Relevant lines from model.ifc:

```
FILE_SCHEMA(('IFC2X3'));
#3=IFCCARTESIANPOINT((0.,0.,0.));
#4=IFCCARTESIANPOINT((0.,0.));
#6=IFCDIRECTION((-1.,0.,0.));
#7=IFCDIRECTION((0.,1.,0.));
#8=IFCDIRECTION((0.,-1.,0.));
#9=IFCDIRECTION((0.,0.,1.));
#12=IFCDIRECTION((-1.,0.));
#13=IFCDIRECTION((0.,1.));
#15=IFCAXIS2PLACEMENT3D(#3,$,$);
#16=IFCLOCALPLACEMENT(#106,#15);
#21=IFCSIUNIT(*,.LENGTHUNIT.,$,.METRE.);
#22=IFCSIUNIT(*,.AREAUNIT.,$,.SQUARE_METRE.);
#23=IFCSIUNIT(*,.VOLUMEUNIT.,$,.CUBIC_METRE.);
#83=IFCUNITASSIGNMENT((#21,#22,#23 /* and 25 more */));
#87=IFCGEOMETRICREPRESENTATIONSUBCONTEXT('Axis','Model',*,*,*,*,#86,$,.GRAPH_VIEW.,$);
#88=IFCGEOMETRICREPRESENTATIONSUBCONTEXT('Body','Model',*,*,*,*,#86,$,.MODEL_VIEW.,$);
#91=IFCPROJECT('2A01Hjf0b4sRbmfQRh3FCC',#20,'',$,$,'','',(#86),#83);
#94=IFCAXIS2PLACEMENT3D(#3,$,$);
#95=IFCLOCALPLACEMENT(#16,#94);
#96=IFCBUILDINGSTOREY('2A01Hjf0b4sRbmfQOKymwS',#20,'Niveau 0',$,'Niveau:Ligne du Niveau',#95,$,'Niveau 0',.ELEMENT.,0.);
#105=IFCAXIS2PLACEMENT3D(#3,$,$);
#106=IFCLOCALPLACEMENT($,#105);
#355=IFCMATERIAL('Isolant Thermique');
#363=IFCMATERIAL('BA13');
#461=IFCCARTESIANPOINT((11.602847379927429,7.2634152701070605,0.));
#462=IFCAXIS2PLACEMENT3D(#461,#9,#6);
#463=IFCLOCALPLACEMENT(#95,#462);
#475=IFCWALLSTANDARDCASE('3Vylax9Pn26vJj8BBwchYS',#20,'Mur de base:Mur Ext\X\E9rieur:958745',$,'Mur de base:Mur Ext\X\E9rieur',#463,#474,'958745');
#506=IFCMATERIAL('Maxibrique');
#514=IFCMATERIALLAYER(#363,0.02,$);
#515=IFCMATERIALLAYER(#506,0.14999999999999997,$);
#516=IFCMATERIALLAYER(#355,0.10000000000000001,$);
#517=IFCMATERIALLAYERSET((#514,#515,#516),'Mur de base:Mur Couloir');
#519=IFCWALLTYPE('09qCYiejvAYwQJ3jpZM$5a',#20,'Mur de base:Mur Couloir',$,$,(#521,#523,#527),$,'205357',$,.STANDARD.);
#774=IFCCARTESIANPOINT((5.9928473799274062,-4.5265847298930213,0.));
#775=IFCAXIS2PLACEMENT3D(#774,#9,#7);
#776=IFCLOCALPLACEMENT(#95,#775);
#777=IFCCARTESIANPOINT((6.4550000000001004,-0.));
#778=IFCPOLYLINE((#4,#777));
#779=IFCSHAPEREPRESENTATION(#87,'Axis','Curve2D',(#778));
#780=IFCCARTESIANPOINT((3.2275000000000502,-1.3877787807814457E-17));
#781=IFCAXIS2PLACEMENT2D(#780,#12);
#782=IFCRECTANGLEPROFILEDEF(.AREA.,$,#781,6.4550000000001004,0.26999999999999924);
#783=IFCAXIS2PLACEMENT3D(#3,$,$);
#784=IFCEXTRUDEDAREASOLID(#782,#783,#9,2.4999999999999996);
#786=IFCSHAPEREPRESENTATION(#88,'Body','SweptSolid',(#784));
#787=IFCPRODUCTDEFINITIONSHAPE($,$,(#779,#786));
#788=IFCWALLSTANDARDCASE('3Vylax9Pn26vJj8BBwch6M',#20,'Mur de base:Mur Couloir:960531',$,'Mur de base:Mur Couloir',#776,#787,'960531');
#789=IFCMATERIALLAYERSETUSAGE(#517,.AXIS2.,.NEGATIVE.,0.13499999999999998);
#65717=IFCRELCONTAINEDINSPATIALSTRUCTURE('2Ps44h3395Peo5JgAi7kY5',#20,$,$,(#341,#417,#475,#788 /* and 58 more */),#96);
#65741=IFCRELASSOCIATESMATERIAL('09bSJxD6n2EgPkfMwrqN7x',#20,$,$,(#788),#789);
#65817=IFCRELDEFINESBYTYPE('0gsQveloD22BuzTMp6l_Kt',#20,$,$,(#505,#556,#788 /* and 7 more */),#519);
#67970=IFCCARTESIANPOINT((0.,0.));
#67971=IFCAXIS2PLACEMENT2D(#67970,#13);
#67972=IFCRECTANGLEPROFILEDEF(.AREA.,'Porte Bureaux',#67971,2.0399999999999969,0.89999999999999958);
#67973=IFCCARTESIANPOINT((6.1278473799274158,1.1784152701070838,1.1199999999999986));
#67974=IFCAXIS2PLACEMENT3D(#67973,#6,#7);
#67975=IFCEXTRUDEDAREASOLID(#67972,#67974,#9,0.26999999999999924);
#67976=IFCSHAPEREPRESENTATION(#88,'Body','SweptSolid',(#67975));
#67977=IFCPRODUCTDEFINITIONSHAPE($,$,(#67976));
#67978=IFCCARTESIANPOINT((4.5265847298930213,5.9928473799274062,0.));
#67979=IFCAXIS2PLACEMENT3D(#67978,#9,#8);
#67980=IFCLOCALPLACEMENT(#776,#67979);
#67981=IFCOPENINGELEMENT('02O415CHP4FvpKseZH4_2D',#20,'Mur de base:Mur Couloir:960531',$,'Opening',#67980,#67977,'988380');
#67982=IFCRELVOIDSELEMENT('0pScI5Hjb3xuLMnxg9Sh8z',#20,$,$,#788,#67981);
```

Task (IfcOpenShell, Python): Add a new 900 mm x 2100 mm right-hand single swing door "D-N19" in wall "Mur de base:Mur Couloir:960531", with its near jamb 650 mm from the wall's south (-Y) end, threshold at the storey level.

```python
import numpy as np
import ifcopenshell
import ifcopenshell.api.feature
import ifcopenshell.api.geometry
import ifcopenshell.api.root
import ifcopenshell.api.spatial
import ifcopenshell.api.type
import ifcopenshell.geom
import ifcopenshell.util.element
import ifcopenshell.util.placement
import ifcopenshell.util.representation
import ifcopenshell.util.shape
import ifcopenshell.util.unit

model = ifcopenshell.open("model.ifc")
unit_scale = ifcopenshell.util.unit.calculate_unit_scale(model)
settings = ifcopenshell.geom.settings()


def volume(element):
    """Net volume in cubic metres, openings subtracted."""
    shape = ifcopenshell.geom.create_shape(settings, element)
    return ifcopenshell.util.shape.get_volume(shape.geometry)


wall = model.by_id(788)
storey = ifcopenshell.util.element.get_container(wall, ifc_class="IfcBuildingStorey")
context = ifcopenshell.util.representation.get_context(model, "Model", "Body", "MODEL_VIEW")
before = volume(wall)

width, height, from_end, sill = 0.9, 2.1, 0.65, 0.0  # metres

# The wall runs along its own X axis, and the end named is its -X end.
wall_shape = ifcopenshell.geom.create_shape(settings, wall)
x, y, z = ifcopenshell.util.shape.get_vertices(wall_shape.geometry).T
start = x.min() + from_end
face, thickness = float(y.min()), float(y.max() - y.min())
wall_matrix = ifcopenshell.util.placement.get_local_placement(wall.ObjectPlacement)
level = ifcopenshell.util.placement.get_local_placement(storey.ObjectPlacement)[2, 3]


def in_wall(x, y):
    """Placement at x, y metres in the wall's axes, at sill height."""
    matrix = wall_matrix.copy()
    matrix[:, 3] = wall_matrix @ np.array([x / unit_scale, y / unit_scale, 0.0, 1.0])
    matrix[2, 3] = level + sill / unit_scale
    return matrix


# Opening: a box that overshoots both wall faces by 50 mm.
opening = ifcopenshell.api.root.create_entity(model, ifc_class="IfcOpeningElement")
box = ifcopenshell.api.geometry.add_wall_representation(
    model, context=context, length=width, height=height, thickness=thickness + 0.1
)
ifcopenshell.api.geometry.assign_representation(model, product=opening, representation=box)
ifcopenshell.api.geometry.edit_object_placement(model, product=opening, matrix=in_wall(start, face - 0.05), is_si=False)
ifcopenshell.api.feature.add_feature(model, feature=opening, element=wall)

door = ifcopenshell.api.root.create_entity(model, ifc_class="IfcDoor", name="D-N19")
door.OverallWidth, door.OverallHeight = width / unit_scale, height / unit_scale
body = ifcopenshell.api.geometry.add_door_representation(
    model,
    context=context,
    overall_width=door.OverallWidth,
    overall_height=door.OverallHeight,
    operation_type="SINGLE_SWING_RIGHT",
    lining_properties={"LiningDepth": thickness / unit_scale, "ThresholdDepth": thickness / unit_scale},
)
ifcopenshell.api.geometry.assign_representation(model, product=door, representation=body)
ifcopenshell.api.spatial.assign_container(model, products=[door], relating_structure=storey)
fills = ifcopenshell.api.feature.add_filling(model, opening=opening, element=door)
fills.OwnerHistory = door.OwnerHistory  # required in IFC2X3

# IFC2X3 keeps the operation on the door style.
style = ifcopenshell.api.root.create_entity(model, ifc_class="IfcDoorStyle", name="D-N19")
style.OperationType, style.ConstructionType = "SINGLE_SWING_RIGHT", "NOTDEFINED"
style.ParameterTakesPrecedence = style.Sizeable = False
ifcopenshell.api.type.assign_type(model, related_objects=[door], relating_type=style)

# The lining spans the wall, so the door starts at the wall face.
ifcopenshell.api.geometry.edit_object_placement(model, product=door, matrix=in_wall(start, face), is_si=False)

after = volume(wall)

print(f"wall volume {before:.3f} -> {after:.3f} m3")

model.write("model_v2.ifc")
```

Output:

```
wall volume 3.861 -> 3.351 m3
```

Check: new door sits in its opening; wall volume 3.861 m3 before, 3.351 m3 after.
